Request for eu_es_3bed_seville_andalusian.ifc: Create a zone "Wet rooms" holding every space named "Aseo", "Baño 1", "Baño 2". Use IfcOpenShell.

First a look at what the model holds.

```python
import ifcopenshell

model = ifcopenshell.open("eu_es_3bed_seville_andalusian.ifc")
print(model.schema)
seen = {}
for space in model.by_type("IfcSpace"):
    seen[space.LongName] = seen.get(space.LongName, 0) + 1
for name, count in sorted(seen.items(), key=str):
    print(count, "x", name)
print("zones:", [z.Name for z in model.by_type("IfcZone")][:20])
```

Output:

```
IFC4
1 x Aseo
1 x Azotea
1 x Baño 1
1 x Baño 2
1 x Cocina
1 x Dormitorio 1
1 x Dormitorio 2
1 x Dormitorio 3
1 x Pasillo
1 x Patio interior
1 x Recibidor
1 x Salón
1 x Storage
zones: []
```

```python
import ifcopenshell
import ifcopenshell.api.group
import ifcopenshell.api.root

model = ifcopenshell.open("eu_es_3bed_seville_andalusian.ifc")

names = {"Aseo", "Baño 1", "Baño 2"}
spaces = [s for s in model.by_type("IfcSpace") if s.LongName in names]

zone = ifcopenshell.api.root.create_entity(model, ifc_class="IfcZone", name="Wet rooms")
ifcopenshell.api.group.assign_group(model, products=spaces, group=zone)
print(len(spaces), "spaces in", zone.Name)

model.write("eu_es_3bed_seville_andalusian_v2.ifc")
```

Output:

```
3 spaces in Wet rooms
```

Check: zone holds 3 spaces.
